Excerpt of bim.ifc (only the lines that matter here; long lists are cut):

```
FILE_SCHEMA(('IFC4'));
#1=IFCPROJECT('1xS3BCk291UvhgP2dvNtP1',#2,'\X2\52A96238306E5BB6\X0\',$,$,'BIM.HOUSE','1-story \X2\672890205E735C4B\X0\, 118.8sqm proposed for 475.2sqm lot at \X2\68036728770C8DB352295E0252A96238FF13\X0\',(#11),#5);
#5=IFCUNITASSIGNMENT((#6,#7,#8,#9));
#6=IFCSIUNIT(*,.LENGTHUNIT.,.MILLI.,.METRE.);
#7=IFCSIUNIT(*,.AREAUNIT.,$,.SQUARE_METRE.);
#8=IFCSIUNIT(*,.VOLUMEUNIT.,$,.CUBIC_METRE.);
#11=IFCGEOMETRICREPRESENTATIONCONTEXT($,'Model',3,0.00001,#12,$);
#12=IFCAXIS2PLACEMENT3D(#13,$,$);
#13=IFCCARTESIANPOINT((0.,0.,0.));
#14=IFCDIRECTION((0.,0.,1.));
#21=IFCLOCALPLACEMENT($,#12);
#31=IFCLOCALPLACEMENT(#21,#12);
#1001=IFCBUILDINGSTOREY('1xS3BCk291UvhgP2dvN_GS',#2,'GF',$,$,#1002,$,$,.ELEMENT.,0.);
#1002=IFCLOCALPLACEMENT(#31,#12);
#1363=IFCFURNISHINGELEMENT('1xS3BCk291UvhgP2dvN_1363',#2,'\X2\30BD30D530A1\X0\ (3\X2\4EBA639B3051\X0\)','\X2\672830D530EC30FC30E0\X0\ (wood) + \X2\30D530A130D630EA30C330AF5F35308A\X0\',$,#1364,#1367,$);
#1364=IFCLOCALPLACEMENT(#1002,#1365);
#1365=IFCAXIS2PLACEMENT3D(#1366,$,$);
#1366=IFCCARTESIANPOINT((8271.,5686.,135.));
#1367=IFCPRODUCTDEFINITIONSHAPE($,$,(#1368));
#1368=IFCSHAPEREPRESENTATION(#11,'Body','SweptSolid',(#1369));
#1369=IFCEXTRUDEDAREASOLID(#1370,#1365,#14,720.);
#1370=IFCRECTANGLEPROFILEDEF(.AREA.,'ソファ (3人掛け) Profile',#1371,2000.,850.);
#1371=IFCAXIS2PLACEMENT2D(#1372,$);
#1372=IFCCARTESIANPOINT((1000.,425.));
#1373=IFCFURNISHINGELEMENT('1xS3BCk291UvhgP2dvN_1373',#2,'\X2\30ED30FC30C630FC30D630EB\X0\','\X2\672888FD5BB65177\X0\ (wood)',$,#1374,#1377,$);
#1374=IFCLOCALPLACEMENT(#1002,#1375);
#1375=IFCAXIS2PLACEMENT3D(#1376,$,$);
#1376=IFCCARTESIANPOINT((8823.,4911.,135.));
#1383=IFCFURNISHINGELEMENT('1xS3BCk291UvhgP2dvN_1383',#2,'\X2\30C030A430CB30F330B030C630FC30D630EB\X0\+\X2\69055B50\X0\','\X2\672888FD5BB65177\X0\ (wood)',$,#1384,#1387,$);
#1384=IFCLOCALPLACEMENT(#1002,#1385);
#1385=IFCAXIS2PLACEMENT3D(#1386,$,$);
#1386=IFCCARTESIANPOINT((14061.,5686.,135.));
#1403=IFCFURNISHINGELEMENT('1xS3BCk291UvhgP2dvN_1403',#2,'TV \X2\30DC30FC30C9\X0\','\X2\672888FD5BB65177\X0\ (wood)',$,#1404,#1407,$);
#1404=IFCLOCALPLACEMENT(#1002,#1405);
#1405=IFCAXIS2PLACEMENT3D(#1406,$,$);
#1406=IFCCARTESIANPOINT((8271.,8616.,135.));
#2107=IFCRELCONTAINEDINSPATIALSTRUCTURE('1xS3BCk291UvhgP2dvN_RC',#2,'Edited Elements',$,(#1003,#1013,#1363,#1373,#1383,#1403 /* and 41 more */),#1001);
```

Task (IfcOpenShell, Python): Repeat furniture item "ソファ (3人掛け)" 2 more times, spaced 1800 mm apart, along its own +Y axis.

```python
import ifcopenshell
import ifcopenshell.api.geometry
import ifcopenshell.api.root
import ifcopenshell.util.element
import ifcopenshell.util.placement

model = ifcopenshell.open("bim.ifc")


def reuse_history(source, copy):
    """copy_class also copies each property set's owner history, people and application; keep the originals."""
    for rel in copy.IsDefinedBy:
        if rel.is_a("IfcRelDefinesByProperties") and (history := rel.RelatingPropertyDefinition.OwnerHistory):
            rel.RelatingPropertyDefinition.OwnerHistory = source.OwnerHistory
            ifcopenshell.util.element.remove_deep2(model, history)


source = model.by_guid("1xS3BCk291UvhgP2dvN_1363")
base = ifcopenshell.util.placement.get_local_placement(source.ObjectPlacement)
step = base[:3, 1] * 1800.0

for i in range(1, 3):
    copy = ifcopenshell.api.root.copy_class(model, product=source)
    copy.Representation = ifcopenshell.util.element.copy_deep(
        model, source.Representation, exclude=["IfcGeometricRepresentationContext", "IfcRepresentationMap"]
    )
    reuse_history(source, copy)
    matrix = base.copy()
    matrix[:3, 3] += i * step
    print("added at", matrix[:3, 3].round(3) + 0.0)
    ifcopenshell.api.geometry.edit_object_placement(model, product=copy, matrix=matrix, is_si=False)

model.write("bim_rev.ifc")
```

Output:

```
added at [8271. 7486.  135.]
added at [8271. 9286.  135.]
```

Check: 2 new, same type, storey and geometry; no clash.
